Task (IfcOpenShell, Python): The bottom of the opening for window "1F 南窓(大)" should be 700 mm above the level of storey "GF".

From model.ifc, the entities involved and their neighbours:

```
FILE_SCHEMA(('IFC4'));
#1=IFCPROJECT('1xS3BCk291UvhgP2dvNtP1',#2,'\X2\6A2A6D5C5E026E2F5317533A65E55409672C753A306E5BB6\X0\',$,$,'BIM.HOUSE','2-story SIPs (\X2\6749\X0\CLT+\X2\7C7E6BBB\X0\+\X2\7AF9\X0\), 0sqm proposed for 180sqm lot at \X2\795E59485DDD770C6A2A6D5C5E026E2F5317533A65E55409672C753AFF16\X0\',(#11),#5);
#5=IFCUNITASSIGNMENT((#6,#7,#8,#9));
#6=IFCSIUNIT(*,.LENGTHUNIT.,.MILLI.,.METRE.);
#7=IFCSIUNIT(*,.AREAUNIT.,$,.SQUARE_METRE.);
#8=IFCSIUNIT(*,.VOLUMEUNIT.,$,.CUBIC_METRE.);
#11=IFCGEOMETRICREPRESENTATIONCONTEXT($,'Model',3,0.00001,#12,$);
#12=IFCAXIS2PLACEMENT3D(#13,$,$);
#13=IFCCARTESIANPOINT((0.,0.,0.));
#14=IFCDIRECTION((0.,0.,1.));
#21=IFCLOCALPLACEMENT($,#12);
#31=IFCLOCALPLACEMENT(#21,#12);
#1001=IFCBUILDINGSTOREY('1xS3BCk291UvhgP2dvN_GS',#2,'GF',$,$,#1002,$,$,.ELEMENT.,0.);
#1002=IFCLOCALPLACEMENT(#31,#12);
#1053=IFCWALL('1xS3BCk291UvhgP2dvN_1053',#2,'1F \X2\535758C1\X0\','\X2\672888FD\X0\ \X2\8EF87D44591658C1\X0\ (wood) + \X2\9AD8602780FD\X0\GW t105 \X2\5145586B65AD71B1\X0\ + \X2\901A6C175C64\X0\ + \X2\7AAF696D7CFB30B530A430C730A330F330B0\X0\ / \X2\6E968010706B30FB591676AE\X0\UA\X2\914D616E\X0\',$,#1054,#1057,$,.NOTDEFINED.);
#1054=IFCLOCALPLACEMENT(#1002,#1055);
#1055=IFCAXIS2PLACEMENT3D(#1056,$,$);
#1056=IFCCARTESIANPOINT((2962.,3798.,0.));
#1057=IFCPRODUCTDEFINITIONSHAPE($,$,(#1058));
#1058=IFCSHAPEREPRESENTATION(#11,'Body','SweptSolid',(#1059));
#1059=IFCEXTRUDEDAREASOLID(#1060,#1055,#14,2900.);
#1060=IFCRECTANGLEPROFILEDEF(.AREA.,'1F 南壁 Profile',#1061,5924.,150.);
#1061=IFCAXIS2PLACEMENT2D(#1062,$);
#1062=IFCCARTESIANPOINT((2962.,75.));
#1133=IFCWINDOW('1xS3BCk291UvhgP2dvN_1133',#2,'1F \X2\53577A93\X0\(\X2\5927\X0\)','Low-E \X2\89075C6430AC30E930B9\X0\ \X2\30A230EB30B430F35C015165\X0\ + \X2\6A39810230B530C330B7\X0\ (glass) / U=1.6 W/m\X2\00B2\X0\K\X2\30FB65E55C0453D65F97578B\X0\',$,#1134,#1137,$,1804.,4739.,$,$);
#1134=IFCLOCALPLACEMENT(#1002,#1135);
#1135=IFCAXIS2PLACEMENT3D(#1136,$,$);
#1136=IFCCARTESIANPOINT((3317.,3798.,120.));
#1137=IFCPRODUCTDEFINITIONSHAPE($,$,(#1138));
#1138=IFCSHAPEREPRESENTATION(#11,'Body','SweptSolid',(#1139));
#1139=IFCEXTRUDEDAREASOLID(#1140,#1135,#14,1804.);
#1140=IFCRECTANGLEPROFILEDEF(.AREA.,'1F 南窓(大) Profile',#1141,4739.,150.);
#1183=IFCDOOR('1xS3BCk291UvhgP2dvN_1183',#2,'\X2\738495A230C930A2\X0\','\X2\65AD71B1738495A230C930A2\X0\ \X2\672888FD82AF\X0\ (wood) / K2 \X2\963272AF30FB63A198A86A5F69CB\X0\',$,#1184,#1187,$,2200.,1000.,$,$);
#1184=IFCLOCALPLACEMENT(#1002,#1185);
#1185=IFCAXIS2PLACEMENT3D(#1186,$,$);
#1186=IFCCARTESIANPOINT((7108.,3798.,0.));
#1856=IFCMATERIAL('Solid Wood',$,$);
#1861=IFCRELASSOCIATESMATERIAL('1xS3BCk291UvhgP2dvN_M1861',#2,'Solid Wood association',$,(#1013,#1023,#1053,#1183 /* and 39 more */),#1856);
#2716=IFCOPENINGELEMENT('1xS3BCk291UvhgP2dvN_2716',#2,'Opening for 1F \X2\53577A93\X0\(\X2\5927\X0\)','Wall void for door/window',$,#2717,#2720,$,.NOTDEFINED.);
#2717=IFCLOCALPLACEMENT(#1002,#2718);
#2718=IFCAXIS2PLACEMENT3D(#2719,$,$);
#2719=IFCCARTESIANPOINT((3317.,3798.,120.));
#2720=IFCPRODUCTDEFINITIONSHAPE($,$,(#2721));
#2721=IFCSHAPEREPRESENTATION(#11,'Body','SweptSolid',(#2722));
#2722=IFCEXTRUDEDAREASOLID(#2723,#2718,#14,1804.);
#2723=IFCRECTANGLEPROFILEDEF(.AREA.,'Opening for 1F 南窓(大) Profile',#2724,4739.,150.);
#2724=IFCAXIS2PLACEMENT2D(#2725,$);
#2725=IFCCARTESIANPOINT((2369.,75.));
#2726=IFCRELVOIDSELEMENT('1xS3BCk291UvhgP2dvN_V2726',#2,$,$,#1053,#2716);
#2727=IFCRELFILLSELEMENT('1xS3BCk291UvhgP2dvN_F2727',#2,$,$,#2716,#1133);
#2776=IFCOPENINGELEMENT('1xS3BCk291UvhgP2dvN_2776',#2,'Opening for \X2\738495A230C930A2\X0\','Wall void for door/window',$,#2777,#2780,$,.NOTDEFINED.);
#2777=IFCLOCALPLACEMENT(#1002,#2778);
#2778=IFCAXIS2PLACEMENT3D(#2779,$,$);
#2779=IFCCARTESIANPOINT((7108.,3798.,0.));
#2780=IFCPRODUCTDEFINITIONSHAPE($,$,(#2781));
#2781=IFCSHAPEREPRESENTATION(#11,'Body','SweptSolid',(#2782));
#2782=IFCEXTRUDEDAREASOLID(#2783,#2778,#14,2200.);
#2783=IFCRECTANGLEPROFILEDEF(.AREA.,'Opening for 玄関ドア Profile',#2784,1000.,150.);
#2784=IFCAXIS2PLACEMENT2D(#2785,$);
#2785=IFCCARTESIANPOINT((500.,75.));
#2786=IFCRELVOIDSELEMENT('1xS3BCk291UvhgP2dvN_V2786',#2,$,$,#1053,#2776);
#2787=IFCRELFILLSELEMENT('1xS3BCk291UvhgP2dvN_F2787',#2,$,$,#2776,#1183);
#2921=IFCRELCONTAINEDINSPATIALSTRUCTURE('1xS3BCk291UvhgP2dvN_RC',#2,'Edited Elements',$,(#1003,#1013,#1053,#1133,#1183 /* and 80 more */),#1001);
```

```python
import numpy as np
import ifcopenshell
import ifcopenshell.api.geometry
import ifcopenshell.geom
import ifcopenshell.util.element
import ifcopenshell.util.placement
import ifcopenshell.util.shape
import ifcopenshell.util.unit

model = ifcopenshell.open("model.ifc")
unit_scale = ifcopenshell.util.unit.calculate_unit_scale(model)

window = model.by_guid("1xS3BCk291UvhgP2dvN_1133")
opening = window.FillsVoids[0].RelatingOpeningElement
storey = ifcopenshell.util.element.get_container(window, ifc_class="IfcBuildingStorey")
level = ifcopenshell.util.placement.get_local_placement(storey.ObjectPlacement)[2, 3]

# The opening's origin need not be at the sill, so measure its lowest point.
shape = ifcopenshell.geom.create_shape(ifcopenshell.geom.settings(), opening)
bottom = ifcopenshell.util.shape.get_shape_bottom_elevation(shape, shape.geometry) / unit_scale
dz = level + 0.7 / unit_scale - bottom

shift = np.array([0.0, 0.0, dz])
# The window is not placed relative to its opening, so move both.
for product in (opening, window):
    matrix = ifcopenshell.util.placement.get_local_placement(product.ObjectPlacement)
    matrix[:3, 3] += shift
    ifcopenshell.api.geometry.edit_object_placement(model, product=product, matrix=matrix, is_si=False)

print(f"moved by {dz * unit_scale:+.3f} m")

model.write("model-out.ifc")
```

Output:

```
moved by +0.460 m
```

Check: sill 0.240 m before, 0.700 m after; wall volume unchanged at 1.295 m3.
